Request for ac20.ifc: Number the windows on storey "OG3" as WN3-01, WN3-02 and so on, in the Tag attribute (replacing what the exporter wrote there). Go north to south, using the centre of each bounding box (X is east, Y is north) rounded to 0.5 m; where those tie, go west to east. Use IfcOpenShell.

First a look at what the model holds.

```python
import ifcopenshell
import ifcopenshell.util.element
import ifcopenshell.util.placement

model = ifcopenshell.open("ac20.ifc")
print(model.schema)
storey = next(s for s in model.by_type("IfcBuildingStorey") if s.Name == "OG3")
windows = [e for e in ifcopenshell.util.element.get_decomposition(storey) if e.is_a("IfcWindow")]
for e in sorted(windows, key=lambda e: e.id()):
    origin = ifcopenshell.util.placement.get_local_placement(e.ObjectPlacement)[:3, 3]
    print(e.id(), e.Tag, e.Name, origin.round(2) + 0.0, sep=" | ")
```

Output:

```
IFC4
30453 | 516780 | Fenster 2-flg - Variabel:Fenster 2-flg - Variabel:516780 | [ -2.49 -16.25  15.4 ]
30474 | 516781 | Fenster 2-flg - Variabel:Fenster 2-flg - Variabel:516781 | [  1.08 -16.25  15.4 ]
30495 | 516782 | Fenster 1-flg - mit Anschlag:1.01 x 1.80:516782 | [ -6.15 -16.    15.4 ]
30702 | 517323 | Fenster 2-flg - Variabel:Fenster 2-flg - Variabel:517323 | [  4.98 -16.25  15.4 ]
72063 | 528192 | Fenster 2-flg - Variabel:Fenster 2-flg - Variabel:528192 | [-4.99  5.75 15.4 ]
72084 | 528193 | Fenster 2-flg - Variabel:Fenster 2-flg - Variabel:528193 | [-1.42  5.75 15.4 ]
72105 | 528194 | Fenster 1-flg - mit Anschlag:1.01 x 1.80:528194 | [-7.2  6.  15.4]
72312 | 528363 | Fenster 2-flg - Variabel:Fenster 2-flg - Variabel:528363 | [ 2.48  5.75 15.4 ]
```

```python
import ifcopenshell
import ifcopenshell.geom
import ifcopenshell.util.element
import ifcopenshell.util.shape

model = ifcopenshell.open("ac20.ifc")
settings = ifcopenshell.geom.settings()
settings.set("use-world-coords", True)


def centre(element):
    shape = ifcopenshell.geom.create_shape(settings, element)
    return ifcopenshell.util.shape.get_bbox_centroid(shape.geometry)


storey = next(s for s in model.by_type("IfcBuildingStorey") if s.Name == "OG3")
windows = [e for e in ifcopenshell.util.element.get_decomposition(storey) if e.is_a("IfcWindow")]

# Insertion points can sit at a corner or the storey origin, so sort by the geometry (in metres).
centres = {e: centre(e) for e in windows}
windows.sort(key=lambda e: (-round(centres[e][1] / 0.5), centres[e][0]))

for i, e in enumerate(windows, start=1):
    number = f"WN3-{i:02d}"
    e.Tag = number
    print(e.id(), number)

model.write("ac20_edited.ifc")
```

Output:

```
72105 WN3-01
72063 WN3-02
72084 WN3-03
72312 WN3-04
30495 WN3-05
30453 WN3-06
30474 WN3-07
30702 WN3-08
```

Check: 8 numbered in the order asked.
